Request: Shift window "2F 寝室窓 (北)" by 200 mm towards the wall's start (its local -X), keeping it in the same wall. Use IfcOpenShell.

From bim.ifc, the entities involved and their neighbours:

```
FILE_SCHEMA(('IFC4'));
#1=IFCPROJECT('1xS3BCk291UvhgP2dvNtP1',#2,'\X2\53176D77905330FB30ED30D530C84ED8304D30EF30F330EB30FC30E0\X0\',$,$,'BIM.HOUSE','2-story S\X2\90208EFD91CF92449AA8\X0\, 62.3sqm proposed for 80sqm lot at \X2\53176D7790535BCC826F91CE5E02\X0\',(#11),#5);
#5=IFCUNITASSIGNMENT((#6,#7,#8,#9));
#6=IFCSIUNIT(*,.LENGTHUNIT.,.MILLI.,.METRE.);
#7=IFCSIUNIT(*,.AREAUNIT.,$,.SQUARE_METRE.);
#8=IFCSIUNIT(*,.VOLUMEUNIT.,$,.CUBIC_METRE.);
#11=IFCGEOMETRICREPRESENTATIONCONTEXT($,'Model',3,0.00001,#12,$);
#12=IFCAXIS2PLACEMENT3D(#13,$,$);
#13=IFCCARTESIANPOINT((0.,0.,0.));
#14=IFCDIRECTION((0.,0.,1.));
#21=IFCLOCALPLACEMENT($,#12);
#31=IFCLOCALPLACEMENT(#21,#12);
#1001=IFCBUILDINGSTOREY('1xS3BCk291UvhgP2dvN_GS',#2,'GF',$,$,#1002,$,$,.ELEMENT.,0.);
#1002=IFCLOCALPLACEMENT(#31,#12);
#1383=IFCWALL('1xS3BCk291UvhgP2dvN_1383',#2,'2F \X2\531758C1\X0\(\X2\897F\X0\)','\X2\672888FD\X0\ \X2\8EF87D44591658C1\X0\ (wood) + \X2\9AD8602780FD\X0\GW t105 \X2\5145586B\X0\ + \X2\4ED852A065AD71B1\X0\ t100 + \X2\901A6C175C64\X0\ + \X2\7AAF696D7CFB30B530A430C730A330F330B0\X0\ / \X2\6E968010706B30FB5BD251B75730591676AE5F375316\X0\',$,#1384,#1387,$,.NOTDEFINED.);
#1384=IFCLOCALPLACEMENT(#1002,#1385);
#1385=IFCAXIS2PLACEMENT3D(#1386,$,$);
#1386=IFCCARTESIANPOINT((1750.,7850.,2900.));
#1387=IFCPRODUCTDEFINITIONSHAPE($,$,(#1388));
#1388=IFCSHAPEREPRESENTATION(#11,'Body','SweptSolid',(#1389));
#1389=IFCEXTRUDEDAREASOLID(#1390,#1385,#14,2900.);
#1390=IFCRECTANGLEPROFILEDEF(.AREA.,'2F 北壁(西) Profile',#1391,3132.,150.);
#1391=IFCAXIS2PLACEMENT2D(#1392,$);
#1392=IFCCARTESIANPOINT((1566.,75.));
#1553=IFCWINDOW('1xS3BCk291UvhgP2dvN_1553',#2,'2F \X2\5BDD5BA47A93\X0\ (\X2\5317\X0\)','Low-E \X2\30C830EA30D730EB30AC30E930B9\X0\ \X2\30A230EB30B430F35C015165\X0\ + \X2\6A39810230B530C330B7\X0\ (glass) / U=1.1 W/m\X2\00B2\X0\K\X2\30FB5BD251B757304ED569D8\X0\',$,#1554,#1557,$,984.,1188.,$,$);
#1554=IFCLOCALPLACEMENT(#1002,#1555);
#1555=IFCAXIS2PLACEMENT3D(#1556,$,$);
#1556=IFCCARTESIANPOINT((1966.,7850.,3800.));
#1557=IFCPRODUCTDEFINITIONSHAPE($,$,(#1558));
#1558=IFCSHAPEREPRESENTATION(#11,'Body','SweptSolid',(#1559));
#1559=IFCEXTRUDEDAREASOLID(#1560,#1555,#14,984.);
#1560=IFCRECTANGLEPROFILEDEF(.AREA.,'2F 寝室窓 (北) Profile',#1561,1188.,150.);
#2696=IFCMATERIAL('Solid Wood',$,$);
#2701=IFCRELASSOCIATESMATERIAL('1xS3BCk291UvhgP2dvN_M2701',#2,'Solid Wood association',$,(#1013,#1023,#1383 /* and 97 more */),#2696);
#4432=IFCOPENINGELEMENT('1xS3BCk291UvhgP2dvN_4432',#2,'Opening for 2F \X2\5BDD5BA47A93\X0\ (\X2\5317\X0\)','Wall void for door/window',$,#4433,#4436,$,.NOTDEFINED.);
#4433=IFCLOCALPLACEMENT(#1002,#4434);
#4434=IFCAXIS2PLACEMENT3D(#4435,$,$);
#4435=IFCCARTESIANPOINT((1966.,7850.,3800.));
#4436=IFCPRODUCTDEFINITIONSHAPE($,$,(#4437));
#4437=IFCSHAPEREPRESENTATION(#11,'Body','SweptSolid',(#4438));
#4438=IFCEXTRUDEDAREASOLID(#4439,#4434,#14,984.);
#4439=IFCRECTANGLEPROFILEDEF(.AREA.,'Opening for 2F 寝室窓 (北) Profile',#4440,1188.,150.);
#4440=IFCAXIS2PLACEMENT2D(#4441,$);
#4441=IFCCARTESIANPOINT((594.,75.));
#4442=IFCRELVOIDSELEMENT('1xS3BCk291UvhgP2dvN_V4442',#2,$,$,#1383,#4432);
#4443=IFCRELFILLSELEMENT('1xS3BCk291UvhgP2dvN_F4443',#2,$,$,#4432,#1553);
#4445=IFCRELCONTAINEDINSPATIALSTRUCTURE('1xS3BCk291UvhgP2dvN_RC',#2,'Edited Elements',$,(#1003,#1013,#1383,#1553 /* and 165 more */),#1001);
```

```python
import ifcopenshell
import ifcopenshell.api.geometry
import ifcopenshell.util.placement
import ifcopenshell.util.unit

model = ifcopenshell.open("bim.ifc")
unit_scale = ifcopenshell.util.unit.calculate_unit_scale(model)

window = model.by_id(1553)
opening = window.FillsVoids[0].RelatingOpeningElement
wall = opening.VoidsElements[0].RelatingBuildingElement

wall_matrix = ifcopenshell.util.placement.get_local_placement(wall.ObjectPlacement)
shift = wall_matrix[:3, 0] * -0.2 / unit_scale
before = ifcopenshell.util.placement.get_local_placement(window.ObjectPlacement)[:3, 3].copy()

# The window is not placed relative to its opening, so move both.
for product in (opening, window):
    matrix = ifcopenshell.util.placement.get_local_placement(product.ObjectPlacement)
    matrix[:3, 3] += shift
    ifcopenshell.api.geometry.edit_object_placement(model, product=product, matrix=matrix, is_si=False)

after = ifcopenshell.util.placement.get_local_placement(window.ObjectPlacement)[:3, 3]
print("window moved by", (after - before).round(3) + 0.0)

model.write("bim_updated.ifc")
```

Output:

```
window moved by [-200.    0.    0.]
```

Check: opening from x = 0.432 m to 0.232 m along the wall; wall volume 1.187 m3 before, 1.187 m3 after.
